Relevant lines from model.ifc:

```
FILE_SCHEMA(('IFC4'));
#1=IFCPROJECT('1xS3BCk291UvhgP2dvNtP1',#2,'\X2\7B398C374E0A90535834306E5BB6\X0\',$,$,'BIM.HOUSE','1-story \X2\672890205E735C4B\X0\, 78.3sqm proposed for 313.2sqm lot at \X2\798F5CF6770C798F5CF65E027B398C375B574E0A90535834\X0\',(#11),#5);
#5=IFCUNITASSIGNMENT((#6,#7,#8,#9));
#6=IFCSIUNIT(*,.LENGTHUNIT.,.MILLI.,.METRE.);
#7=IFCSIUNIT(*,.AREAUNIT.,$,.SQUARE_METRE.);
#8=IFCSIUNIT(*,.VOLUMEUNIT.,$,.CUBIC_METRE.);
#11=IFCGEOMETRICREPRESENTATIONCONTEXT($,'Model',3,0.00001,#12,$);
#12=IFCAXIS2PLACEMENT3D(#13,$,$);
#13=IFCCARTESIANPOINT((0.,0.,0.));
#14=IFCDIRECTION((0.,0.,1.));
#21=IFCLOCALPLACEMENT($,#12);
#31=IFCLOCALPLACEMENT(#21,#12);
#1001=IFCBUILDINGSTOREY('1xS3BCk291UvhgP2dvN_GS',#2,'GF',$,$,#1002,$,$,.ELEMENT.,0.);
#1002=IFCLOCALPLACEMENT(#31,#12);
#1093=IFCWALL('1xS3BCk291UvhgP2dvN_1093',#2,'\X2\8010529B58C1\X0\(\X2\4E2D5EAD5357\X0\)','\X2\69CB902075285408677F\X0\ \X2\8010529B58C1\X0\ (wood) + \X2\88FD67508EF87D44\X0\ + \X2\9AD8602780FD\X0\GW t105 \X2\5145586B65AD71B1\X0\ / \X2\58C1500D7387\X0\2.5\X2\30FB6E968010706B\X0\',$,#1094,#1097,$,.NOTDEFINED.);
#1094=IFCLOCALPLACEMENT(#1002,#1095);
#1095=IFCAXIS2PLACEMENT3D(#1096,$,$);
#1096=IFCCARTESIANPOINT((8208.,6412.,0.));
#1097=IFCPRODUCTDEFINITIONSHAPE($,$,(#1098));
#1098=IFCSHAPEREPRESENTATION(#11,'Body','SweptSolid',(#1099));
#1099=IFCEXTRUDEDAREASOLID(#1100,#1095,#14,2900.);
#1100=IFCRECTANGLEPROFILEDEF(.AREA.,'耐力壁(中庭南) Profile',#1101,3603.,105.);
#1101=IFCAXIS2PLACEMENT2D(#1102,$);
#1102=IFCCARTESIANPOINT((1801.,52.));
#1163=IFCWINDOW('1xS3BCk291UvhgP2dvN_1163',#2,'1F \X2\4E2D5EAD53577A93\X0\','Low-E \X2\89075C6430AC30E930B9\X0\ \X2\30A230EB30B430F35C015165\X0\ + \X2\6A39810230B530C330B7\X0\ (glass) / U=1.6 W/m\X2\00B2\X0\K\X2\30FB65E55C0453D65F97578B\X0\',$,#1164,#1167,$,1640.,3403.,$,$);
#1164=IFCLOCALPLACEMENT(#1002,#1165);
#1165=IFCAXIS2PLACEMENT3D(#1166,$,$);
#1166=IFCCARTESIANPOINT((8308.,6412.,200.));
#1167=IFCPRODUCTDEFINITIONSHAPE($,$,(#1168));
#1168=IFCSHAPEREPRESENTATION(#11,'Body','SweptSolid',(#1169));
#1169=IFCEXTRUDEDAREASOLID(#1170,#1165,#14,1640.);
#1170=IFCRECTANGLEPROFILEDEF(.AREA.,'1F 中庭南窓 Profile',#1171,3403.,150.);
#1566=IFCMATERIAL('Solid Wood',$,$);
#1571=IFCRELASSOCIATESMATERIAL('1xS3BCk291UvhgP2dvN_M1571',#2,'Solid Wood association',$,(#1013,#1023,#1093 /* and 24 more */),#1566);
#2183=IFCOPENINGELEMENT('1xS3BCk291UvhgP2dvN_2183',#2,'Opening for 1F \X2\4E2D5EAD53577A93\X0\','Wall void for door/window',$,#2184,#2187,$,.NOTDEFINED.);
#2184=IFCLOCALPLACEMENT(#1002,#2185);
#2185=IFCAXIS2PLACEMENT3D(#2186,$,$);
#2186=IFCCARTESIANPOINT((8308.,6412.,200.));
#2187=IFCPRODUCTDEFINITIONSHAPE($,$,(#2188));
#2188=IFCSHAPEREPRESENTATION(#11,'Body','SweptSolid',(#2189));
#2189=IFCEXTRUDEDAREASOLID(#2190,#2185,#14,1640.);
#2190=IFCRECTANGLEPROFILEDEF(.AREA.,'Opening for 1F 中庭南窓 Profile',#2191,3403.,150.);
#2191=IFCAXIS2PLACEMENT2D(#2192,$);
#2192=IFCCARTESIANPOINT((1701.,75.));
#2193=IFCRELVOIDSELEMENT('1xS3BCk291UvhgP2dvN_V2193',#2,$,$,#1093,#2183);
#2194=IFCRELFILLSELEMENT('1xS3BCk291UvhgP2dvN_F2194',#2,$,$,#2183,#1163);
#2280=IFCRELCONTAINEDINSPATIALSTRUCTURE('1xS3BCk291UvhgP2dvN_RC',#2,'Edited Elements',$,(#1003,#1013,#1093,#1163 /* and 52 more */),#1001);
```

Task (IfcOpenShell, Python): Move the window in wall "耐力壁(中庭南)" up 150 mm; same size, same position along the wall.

```python
import numpy as np
import ifcopenshell
import ifcopenshell.api.geometry
import ifcopenshell.util.placement
import ifcopenshell.util.unit

model = ifcopenshell.open("model.ifc")
unit_scale = ifcopenshell.util.unit.calculate_unit_scale(model)

window = model.by_guid("1xS3BCk291UvhgP2dvN_1163")
opening = window.FillsVoids[0].RelatingOpeningElement
dz = 150.0

shift = np.array([0.0, 0.0, dz])
# The window is not placed relative to its opening, so move both.
for product in (opening, window):
    matrix = ifcopenshell.util.placement.get_local_placement(product.ObjectPlacement)
    matrix[:3, 3] += shift
    ifcopenshell.api.geometry.edit_object_placement(model, product=product, matrix=matrix, is_si=False)

print(f"moved by {dz * unit_scale:+.3f} m")

model.write("model-out.ifc")
```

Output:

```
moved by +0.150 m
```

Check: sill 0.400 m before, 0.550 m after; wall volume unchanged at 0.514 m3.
